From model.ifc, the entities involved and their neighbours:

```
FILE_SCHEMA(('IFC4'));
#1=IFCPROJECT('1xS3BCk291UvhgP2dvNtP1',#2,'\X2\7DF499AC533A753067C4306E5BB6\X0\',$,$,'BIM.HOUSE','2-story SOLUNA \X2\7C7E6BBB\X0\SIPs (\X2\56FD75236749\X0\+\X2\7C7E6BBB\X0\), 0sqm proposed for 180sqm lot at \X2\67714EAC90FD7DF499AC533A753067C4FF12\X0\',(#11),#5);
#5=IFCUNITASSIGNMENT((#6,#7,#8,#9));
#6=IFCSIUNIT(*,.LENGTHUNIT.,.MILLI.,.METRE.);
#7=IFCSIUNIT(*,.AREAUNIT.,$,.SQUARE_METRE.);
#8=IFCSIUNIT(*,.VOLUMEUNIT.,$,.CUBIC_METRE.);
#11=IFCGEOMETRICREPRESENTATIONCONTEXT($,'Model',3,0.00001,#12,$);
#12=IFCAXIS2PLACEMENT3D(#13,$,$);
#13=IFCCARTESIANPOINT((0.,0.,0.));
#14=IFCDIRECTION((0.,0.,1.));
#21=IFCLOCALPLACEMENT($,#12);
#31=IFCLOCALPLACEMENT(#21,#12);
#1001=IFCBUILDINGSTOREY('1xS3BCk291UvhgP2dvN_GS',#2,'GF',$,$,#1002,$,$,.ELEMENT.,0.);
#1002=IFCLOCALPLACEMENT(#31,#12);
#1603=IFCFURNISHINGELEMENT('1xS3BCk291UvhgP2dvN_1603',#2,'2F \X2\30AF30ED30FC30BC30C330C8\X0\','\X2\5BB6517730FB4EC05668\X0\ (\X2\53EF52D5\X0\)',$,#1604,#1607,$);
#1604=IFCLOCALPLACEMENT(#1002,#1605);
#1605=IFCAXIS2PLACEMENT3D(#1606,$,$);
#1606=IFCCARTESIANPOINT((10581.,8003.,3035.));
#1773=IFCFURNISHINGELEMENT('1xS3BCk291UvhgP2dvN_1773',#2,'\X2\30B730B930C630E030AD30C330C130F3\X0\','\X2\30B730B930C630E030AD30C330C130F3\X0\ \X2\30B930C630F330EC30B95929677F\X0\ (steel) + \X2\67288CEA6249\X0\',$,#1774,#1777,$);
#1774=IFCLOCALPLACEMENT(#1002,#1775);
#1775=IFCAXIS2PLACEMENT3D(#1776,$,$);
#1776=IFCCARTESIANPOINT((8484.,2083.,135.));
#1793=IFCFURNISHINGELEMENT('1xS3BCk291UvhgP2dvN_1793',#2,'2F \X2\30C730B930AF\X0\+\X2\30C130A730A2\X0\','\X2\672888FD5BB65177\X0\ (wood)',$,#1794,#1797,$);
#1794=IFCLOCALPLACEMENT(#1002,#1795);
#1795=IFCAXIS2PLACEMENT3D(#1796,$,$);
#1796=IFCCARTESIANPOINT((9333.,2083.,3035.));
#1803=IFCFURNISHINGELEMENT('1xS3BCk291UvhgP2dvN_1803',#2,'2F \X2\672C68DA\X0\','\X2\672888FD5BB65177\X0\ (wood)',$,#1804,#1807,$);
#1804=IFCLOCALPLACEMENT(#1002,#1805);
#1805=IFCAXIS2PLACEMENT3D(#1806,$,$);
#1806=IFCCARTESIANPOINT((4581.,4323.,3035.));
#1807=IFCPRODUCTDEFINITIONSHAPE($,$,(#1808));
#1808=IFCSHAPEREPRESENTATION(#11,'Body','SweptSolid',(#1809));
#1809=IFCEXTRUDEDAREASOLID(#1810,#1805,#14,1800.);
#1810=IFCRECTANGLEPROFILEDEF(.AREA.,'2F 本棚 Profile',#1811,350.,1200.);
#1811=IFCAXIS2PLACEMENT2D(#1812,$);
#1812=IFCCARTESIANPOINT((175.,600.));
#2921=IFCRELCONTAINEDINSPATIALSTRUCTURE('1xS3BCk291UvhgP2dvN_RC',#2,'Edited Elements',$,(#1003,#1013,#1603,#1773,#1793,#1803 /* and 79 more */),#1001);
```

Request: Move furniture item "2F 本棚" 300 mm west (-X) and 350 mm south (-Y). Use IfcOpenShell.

```python
import ifcopenshell
import ifcopenshell.api.geometry
import ifcopenshell.util.placement
import ifcopenshell.util.unit

model = ifcopenshell.open("model.ifc")
unit_scale = ifcopenshell.util.unit.calculate_unit_scale(model)

item = model.by_guid("1xS3BCk291UvhgP2dvN_1803")
matrix = ifcopenshell.util.placement.get_local_placement(item.ObjectPlacement)
matrix[0, 3] -= 0.3 / unit_scale
matrix[1, 3] -= 0.35 / unit_scale
ifcopenshell.api.geometry.edit_object_placement(model, product=item, matrix=matrix, is_si=False)

print(ifcopenshell.util.placement.get_local_placement(item.ObjectPlacement).round(3) + 0.0)

model.write("model_edited.ifc")
```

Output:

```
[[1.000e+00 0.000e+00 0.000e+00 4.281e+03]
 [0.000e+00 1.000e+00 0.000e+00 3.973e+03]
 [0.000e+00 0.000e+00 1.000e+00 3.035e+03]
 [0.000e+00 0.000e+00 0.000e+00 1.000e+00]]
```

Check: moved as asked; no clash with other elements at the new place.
